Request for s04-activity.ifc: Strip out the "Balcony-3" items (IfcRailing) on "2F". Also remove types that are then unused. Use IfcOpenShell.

First a look at what the model holds.

```python
import ifcopenshell
import ifcopenshell.util.element

model = ifcopenshell.open("s04-activity.ifc")
print(model.schema)
storey = next(s for s in model.by_type("IfcBuildingStorey") if s.Name == "2F")
railings = [e for e in ifcopenshell.util.element.get_decomposition(storey) if e.is_a("IfcRailing")]
seen = {}
for e in railings:
    element_type = ifcopenshell.util.element.get_type(e)
    name = element_type.Name if element_type not in (None, e) else None
    seen[name] = seen.get(name, 0) + 1
for name, count in sorted(seen.items(), key=str):
    print(count, "x", name)
```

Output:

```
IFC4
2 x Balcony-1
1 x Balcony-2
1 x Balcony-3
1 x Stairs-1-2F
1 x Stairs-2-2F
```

```python
import ifcopenshell
import ifcopenshell.api.root
import ifcopenshell.util.element

model = ifcopenshell.open("s04-activity.ifc")

storey = next(s for s in model.by_type("IfcBuildingStorey") if s.Name == "2F")
railings = [e for e in ifcopenshell.util.element.get_decomposition(storey) if e.is_a("IfcRailing")]
targets = [e for e in railings if (t := ifcopenshell.util.element.get_type(e)) not in (None, e) and t.Name == "Balcony-3"]
types = {ifcopenshell.util.element.get_type(e) for e in targets} - {None, *targets}

for e in targets:
    ifcopenshell.api.root.remove_product(model, product=e)
print(len(targets), "removed")

unused = [t for t in types if not ifcopenshell.util.element.get_types(t)]
for t in unused:
    ifcopenshell.api.root.remove_product(model, product=t)
print(len(unused), "unused types removed")

model.write("s04-activity_updated.ifc")
```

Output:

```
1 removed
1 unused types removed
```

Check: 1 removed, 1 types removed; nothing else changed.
